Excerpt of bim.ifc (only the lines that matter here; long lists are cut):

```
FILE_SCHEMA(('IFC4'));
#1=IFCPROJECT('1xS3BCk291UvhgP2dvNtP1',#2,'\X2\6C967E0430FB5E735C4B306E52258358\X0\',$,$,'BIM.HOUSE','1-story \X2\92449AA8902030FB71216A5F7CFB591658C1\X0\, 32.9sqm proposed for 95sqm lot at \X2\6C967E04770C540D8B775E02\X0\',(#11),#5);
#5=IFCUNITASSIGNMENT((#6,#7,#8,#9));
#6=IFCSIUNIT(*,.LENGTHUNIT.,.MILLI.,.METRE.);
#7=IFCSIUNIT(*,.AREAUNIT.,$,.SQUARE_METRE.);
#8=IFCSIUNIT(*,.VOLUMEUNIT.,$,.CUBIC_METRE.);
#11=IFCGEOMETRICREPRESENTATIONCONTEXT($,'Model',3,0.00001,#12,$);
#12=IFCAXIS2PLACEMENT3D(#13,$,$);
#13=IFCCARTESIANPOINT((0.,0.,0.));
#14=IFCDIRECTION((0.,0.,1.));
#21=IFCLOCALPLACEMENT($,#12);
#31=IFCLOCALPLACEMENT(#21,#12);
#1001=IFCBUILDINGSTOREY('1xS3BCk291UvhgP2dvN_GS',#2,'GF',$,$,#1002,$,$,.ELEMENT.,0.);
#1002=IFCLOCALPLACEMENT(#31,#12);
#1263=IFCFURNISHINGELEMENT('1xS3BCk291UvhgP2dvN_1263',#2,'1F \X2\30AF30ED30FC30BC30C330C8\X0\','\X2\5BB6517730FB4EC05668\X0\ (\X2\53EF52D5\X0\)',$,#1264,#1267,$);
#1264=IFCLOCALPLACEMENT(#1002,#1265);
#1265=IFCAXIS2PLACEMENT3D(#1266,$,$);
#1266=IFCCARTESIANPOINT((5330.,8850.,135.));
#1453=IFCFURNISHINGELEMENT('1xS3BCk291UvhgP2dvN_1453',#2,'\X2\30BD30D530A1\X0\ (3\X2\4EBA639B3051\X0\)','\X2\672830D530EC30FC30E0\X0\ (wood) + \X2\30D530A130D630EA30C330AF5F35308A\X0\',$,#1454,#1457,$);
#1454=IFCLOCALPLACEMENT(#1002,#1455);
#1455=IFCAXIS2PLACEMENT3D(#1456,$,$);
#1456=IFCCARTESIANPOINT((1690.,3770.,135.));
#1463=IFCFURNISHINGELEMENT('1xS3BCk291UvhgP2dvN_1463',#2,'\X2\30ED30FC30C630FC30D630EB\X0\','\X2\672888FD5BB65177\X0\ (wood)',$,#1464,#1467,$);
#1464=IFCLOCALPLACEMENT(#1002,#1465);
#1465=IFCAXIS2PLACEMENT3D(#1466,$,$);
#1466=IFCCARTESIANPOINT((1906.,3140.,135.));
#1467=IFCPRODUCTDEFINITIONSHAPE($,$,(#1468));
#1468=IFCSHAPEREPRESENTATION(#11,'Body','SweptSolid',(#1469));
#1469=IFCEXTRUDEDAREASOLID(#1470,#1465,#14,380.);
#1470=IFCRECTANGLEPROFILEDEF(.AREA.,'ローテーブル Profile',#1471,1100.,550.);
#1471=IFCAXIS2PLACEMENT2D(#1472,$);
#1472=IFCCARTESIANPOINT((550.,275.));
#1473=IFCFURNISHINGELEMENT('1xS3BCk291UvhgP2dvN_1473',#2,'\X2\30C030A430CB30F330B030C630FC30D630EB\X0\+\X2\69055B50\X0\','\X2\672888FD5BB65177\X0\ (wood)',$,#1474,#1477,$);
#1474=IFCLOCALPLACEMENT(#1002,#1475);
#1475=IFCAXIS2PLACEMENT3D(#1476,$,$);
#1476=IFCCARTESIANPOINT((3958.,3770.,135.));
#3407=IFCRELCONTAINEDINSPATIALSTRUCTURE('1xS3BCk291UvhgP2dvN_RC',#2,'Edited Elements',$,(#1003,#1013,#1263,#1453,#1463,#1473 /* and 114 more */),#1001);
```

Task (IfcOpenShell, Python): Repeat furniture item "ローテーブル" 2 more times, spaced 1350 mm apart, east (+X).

```python
import numpy as np
import ifcopenshell
import ifcopenshell.api.geometry
import ifcopenshell.api.root
import ifcopenshell.util.element
import ifcopenshell.util.placement

model = ifcopenshell.open("bim.ifc")


def reuse_history(source, copy):
    """copy_class also copies each property set's owner history, people and application; keep the originals."""
    for rel in copy.IsDefinedBy:
        if rel.is_a("IfcRelDefinesByProperties") and (history := rel.RelatingPropertyDefinition.OwnerHistory):
            rel.RelatingPropertyDefinition.OwnerHistory = source.OwnerHistory
            ifcopenshell.util.element.remove_deep2(model, history)


source = model.by_guid("1xS3BCk291UvhgP2dvN_1463")
base = ifcopenshell.util.placement.get_local_placement(source.ObjectPlacement)
step = np.array([1.0, 0.0, 0.0]) * 1350.0

for i in range(1, 3):
    copy = ifcopenshell.api.root.copy_class(model, product=source)
    copy.Representation = ifcopenshell.util.element.copy_deep(
        model, source.Representation, exclude=["IfcGeometricRepresentationContext", "IfcRepresentationMap"]
    )
    reuse_history(source, copy)
    matrix = base.copy()
    matrix[:3, 3] += i * step
    print("added at", matrix[:3, 3].round(3) + 0.0)
    ifcopenshell.api.geometry.edit_object_placement(model, product=copy, matrix=matrix, is_si=False)

model.write("bim_updated.ifc")
```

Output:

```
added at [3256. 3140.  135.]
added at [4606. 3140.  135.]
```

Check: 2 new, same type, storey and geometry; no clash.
